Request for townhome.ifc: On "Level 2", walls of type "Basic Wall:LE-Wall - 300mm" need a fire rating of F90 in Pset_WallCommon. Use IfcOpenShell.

First a look at what the model holds.

```python
import ifcopenshell
import ifcopenshell.util.element

model = ifcopenshell.open("townhome.ifc")
print(model.schema)
storey = next(s for s in model.by_type("IfcBuildingStorey") if s.Name == "Level 2")
walls = [e for e in ifcopenshell.util.element.get_decomposition(storey) if e.is_a("IfcWall")]
seen = {}
for e in walls:
    element_type = ifcopenshell.util.element.get_type(e)
    key = (element_type.Name if element_type != e and element_type else None, ifcopenshell.util.element.get_pset(e, "Pset_WallCommon", "FireRating"))
    seen[key] = seen.get(key, 0) + 1
for (name, value), count in sorted(seen.items(), key=str):
    print(count, "x", name, "|", value)
```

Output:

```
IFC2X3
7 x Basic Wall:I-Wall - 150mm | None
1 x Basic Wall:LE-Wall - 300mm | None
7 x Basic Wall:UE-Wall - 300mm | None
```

```python
import ifcopenshell
import ifcopenshell.api.pset
import ifcopenshell.util.element

model = ifcopenshell.open("townhome.ifc")

storey = next(s for s in model.by_type("IfcBuildingStorey") if s.Name == "Level 2")
walls = [e for e in ifcopenshell.util.element.get_decomposition(storey) if e.is_a("IfcWall")]

count = 0
for e in walls:
    element_type = ifcopenshell.util.element.get_type(e)
    if element_type in (None, e) or element_type.Name != "Basic Wall:LE-Wall - 300mm":
        continue
    # add_pset returns the element's existing set when there is one.
    pset = ifcopenshell.api.pset.add_pset(model, product=e, name="Pset_WallCommon")
    ifcopenshell.api.pset.edit_pset(model, pset=pset, properties={"FireRating": "F90"})
    count += 1

print(count, "walls updated")

model.write("townhome_edited.ifc")
```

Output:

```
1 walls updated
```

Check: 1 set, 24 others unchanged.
